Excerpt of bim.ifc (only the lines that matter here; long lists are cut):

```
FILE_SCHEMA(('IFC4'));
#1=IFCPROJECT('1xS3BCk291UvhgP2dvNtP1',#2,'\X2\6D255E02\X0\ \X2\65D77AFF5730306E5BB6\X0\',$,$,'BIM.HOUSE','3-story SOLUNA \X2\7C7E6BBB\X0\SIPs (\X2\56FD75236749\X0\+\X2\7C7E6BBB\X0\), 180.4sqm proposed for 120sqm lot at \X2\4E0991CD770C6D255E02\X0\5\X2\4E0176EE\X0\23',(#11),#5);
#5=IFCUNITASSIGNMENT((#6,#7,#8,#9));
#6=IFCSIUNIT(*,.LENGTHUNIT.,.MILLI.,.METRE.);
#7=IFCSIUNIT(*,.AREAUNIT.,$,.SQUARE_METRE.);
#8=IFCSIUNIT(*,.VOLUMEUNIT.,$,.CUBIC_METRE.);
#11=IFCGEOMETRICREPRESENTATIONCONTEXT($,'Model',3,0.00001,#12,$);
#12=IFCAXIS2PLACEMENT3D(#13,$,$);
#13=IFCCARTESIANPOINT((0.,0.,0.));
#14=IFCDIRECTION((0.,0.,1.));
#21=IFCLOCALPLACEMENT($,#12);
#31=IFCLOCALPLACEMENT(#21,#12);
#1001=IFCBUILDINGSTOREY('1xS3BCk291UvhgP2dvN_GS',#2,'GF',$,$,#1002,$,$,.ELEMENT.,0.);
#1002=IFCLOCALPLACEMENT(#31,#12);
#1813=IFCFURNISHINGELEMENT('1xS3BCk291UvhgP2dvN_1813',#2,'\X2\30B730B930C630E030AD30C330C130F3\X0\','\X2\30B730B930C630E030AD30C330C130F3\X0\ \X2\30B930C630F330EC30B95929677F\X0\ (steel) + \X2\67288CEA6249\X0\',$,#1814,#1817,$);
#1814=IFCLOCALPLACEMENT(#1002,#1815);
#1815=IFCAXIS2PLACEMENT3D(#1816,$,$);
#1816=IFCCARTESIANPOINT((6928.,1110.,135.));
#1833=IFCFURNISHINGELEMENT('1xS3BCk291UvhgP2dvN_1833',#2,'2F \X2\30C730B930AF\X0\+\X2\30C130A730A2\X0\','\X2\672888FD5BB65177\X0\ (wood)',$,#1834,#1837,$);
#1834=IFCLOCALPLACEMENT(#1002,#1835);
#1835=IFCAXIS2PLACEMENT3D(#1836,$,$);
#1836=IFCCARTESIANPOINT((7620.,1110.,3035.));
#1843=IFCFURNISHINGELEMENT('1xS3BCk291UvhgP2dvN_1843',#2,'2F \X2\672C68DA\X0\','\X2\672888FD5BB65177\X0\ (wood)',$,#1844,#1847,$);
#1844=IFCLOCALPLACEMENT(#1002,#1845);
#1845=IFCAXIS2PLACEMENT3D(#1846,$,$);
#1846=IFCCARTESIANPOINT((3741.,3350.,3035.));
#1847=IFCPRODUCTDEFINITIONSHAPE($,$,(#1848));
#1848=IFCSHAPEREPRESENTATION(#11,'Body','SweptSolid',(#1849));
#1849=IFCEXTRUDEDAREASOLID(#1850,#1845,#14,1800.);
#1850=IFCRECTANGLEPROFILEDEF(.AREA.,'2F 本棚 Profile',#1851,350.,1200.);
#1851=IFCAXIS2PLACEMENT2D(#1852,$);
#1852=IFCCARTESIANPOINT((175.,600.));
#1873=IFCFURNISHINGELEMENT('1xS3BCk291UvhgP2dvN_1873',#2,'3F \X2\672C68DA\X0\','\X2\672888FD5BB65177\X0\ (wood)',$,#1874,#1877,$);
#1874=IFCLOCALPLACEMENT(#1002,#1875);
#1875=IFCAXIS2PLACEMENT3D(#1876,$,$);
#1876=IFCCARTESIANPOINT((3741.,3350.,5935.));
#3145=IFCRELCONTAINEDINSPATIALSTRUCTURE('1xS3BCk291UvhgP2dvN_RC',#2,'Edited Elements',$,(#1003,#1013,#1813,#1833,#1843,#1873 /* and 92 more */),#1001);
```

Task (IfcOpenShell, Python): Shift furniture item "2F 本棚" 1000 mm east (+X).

```python
import ifcopenshell
import ifcopenshell.api.geometry
import ifcopenshell.util.placement
import ifcopenshell.util.unit

model = ifcopenshell.open("bim.ifc")
unit_scale = ifcopenshell.util.unit.calculate_unit_scale(model)

item = model.by_guid("1xS3BCk291UvhgP2dvN_1843")
matrix = ifcopenshell.util.placement.get_local_placement(item.ObjectPlacement)
matrix[0, 3] += 1 / unit_scale
ifcopenshell.api.geometry.edit_object_placement(model, product=item, matrix=matrix, is_si=False)

print(ifcopenshell.util.placement.get_local_placement(item.ObjectPlacement).round(3) + 0.0)

model.write("bim_v2.ifc")
```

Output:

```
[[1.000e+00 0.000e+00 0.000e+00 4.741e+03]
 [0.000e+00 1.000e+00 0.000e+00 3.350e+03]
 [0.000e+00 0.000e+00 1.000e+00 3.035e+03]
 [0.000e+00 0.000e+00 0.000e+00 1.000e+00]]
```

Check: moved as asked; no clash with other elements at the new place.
